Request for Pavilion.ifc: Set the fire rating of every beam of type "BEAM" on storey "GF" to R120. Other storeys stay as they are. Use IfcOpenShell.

First a look at what the model holds.

```python
import ifcopenshell
import ifcopenshell.util.element

model = ifcopenshell.open("Pavilion.ifc")
print(model.schema)
storey = next(s for s in model.by_type("IfcBuildingStorey") if s.Name == "GF")
beams = [e for e in ifcopenshell.util.element.get_decomposition(storey) if e.is_a("IfcBeam")]
seen = {}
for e in beams:
    element_type = ifcopenshell.util.element.get_type(e)
    key = (element_type.Name if element_type != e and element_type else None, ifcopenshell.util.element.get_pset(e, "Pset_BeamCommon", "FireRating"))
    seen[key] = seen.get(key, 0) + 1
for (name, value), count in sorted(seen.items(), key=str):
    print(count, "x", name, "|", value)
```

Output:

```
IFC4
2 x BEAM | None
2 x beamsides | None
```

```python
import ifcopenshell
import ifcopenshell.api.pset
import ifcopenshell.util.element

model = ifcopenshell.open("Pavilion.ifc")

storey = next(s for s in model.by_type("IfcBuildingStorey") if s.Name == "GF")
beams = [e for e in ifcopenshell.util.element.get_decomposition(storey) if e.is_a("IfcBeam")]

count = 0
for e in beams:
    element_type = ifcopenshell.util.element.get_type(e)
    if element_type in (None, e) or element_type.Name != "BEAM":
        continue
    # add_pset returns the element's existing set when there is one.
    pset = ifcopenshell.api.pset.add_pset(model, product=e, name="Pset_BeamCommon")
    ifcopenshell.api.pset.edit_pset(model, pset=pset, properties={"FireRating": "R120"})
    count += 1

print(count, "beams updated")

model.write("Pavilion_edited.ifc")
```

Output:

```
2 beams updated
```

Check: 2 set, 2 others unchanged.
